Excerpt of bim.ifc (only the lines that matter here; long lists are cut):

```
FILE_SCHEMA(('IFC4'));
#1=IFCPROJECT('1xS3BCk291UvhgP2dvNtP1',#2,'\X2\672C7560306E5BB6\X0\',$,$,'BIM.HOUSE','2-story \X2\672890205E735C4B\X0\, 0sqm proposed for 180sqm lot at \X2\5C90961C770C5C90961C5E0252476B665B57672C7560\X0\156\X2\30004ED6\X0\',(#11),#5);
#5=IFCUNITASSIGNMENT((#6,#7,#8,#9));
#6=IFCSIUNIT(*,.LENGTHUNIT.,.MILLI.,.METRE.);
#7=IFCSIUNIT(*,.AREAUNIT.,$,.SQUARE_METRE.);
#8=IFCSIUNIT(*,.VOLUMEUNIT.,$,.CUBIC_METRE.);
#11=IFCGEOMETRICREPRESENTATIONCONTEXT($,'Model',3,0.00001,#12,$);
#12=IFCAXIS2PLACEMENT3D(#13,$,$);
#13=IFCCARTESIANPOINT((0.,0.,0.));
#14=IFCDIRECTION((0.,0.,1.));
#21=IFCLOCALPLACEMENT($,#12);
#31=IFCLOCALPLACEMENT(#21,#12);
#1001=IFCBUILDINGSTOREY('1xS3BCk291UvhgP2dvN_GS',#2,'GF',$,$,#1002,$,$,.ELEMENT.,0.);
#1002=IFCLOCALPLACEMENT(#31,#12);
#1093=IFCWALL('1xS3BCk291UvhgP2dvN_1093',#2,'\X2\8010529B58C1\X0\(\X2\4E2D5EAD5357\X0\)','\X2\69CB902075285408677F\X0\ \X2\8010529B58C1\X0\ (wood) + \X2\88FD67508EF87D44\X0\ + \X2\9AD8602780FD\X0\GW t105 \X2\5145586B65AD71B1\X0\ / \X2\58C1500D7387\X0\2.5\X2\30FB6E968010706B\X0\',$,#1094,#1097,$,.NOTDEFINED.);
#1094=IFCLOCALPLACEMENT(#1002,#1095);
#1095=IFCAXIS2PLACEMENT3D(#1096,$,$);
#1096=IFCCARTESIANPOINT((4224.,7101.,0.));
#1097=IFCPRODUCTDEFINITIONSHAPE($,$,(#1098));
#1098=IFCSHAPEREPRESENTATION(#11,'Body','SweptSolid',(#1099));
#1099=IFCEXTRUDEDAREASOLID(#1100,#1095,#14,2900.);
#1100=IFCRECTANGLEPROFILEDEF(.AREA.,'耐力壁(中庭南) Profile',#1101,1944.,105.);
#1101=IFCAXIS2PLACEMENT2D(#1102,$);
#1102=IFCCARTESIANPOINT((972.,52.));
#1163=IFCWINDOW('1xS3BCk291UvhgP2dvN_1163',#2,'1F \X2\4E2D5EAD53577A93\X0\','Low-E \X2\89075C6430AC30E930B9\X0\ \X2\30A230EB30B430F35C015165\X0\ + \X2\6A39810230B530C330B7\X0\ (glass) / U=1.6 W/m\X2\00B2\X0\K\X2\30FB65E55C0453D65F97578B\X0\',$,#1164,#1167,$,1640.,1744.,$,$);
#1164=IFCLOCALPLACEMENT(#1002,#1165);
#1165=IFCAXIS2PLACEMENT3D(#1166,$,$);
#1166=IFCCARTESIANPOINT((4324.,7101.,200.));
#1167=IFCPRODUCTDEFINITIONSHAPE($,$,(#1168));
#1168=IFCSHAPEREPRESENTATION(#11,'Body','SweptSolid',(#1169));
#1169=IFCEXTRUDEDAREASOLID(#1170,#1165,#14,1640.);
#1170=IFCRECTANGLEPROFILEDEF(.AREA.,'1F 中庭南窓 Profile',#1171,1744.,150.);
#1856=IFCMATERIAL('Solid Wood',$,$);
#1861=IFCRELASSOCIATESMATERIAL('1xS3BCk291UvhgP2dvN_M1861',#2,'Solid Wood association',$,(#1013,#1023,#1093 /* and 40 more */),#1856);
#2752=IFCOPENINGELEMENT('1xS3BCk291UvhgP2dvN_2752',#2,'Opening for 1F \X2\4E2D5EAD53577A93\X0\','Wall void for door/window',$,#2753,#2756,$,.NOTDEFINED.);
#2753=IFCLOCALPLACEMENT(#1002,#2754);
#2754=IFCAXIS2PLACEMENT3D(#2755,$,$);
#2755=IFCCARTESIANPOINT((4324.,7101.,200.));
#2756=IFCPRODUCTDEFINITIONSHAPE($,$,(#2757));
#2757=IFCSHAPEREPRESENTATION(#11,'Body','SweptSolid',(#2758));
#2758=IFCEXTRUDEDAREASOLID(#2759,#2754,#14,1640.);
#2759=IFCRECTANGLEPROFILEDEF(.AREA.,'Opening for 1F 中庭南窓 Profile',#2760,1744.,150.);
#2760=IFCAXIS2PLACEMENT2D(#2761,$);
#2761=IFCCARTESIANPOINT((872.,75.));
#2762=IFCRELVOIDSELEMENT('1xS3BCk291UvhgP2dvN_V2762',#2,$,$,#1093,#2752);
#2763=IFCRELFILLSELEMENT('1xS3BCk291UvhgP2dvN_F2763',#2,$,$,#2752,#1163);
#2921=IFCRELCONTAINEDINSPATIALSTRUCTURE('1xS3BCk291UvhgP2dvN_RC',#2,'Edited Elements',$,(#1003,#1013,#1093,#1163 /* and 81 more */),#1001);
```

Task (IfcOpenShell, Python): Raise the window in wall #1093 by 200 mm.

```python
import numpy as np
import ifcopenshell
import ifcopenshell.api.geometry
import ifcopenshell.util.placement
import ifcopenshell.util.unit

model = ifcopenshell.open("bim.ifc")
unit_scale = ifcopenshell.util.unit.calculate_unit_scale(model)

window = model.by_guid("1xS3BCk291UvhgP2dvN_1163")
opening = window.FillsVoids[0].RelatingOpeningElement
dz = 200.0

shift = np.array([0.0, 0.0, dz])
# The window is not placed relative to its opening, so move both.
for product in (opening, window):
    matrix = ifcopenshell.util.placement.get_local_placement(product.ObjectPlacement)
    matrix[:3, 3] += shift
    ifcopenshell.api.geometry.edit_object_placement(model, product=product, matrix=matrix, is_si=False)

print(f"moved by {dz * unit_scale:+.3f} m")

model.write("bim_v2.ifc")
```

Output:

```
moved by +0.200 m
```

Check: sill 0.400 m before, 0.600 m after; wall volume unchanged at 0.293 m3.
